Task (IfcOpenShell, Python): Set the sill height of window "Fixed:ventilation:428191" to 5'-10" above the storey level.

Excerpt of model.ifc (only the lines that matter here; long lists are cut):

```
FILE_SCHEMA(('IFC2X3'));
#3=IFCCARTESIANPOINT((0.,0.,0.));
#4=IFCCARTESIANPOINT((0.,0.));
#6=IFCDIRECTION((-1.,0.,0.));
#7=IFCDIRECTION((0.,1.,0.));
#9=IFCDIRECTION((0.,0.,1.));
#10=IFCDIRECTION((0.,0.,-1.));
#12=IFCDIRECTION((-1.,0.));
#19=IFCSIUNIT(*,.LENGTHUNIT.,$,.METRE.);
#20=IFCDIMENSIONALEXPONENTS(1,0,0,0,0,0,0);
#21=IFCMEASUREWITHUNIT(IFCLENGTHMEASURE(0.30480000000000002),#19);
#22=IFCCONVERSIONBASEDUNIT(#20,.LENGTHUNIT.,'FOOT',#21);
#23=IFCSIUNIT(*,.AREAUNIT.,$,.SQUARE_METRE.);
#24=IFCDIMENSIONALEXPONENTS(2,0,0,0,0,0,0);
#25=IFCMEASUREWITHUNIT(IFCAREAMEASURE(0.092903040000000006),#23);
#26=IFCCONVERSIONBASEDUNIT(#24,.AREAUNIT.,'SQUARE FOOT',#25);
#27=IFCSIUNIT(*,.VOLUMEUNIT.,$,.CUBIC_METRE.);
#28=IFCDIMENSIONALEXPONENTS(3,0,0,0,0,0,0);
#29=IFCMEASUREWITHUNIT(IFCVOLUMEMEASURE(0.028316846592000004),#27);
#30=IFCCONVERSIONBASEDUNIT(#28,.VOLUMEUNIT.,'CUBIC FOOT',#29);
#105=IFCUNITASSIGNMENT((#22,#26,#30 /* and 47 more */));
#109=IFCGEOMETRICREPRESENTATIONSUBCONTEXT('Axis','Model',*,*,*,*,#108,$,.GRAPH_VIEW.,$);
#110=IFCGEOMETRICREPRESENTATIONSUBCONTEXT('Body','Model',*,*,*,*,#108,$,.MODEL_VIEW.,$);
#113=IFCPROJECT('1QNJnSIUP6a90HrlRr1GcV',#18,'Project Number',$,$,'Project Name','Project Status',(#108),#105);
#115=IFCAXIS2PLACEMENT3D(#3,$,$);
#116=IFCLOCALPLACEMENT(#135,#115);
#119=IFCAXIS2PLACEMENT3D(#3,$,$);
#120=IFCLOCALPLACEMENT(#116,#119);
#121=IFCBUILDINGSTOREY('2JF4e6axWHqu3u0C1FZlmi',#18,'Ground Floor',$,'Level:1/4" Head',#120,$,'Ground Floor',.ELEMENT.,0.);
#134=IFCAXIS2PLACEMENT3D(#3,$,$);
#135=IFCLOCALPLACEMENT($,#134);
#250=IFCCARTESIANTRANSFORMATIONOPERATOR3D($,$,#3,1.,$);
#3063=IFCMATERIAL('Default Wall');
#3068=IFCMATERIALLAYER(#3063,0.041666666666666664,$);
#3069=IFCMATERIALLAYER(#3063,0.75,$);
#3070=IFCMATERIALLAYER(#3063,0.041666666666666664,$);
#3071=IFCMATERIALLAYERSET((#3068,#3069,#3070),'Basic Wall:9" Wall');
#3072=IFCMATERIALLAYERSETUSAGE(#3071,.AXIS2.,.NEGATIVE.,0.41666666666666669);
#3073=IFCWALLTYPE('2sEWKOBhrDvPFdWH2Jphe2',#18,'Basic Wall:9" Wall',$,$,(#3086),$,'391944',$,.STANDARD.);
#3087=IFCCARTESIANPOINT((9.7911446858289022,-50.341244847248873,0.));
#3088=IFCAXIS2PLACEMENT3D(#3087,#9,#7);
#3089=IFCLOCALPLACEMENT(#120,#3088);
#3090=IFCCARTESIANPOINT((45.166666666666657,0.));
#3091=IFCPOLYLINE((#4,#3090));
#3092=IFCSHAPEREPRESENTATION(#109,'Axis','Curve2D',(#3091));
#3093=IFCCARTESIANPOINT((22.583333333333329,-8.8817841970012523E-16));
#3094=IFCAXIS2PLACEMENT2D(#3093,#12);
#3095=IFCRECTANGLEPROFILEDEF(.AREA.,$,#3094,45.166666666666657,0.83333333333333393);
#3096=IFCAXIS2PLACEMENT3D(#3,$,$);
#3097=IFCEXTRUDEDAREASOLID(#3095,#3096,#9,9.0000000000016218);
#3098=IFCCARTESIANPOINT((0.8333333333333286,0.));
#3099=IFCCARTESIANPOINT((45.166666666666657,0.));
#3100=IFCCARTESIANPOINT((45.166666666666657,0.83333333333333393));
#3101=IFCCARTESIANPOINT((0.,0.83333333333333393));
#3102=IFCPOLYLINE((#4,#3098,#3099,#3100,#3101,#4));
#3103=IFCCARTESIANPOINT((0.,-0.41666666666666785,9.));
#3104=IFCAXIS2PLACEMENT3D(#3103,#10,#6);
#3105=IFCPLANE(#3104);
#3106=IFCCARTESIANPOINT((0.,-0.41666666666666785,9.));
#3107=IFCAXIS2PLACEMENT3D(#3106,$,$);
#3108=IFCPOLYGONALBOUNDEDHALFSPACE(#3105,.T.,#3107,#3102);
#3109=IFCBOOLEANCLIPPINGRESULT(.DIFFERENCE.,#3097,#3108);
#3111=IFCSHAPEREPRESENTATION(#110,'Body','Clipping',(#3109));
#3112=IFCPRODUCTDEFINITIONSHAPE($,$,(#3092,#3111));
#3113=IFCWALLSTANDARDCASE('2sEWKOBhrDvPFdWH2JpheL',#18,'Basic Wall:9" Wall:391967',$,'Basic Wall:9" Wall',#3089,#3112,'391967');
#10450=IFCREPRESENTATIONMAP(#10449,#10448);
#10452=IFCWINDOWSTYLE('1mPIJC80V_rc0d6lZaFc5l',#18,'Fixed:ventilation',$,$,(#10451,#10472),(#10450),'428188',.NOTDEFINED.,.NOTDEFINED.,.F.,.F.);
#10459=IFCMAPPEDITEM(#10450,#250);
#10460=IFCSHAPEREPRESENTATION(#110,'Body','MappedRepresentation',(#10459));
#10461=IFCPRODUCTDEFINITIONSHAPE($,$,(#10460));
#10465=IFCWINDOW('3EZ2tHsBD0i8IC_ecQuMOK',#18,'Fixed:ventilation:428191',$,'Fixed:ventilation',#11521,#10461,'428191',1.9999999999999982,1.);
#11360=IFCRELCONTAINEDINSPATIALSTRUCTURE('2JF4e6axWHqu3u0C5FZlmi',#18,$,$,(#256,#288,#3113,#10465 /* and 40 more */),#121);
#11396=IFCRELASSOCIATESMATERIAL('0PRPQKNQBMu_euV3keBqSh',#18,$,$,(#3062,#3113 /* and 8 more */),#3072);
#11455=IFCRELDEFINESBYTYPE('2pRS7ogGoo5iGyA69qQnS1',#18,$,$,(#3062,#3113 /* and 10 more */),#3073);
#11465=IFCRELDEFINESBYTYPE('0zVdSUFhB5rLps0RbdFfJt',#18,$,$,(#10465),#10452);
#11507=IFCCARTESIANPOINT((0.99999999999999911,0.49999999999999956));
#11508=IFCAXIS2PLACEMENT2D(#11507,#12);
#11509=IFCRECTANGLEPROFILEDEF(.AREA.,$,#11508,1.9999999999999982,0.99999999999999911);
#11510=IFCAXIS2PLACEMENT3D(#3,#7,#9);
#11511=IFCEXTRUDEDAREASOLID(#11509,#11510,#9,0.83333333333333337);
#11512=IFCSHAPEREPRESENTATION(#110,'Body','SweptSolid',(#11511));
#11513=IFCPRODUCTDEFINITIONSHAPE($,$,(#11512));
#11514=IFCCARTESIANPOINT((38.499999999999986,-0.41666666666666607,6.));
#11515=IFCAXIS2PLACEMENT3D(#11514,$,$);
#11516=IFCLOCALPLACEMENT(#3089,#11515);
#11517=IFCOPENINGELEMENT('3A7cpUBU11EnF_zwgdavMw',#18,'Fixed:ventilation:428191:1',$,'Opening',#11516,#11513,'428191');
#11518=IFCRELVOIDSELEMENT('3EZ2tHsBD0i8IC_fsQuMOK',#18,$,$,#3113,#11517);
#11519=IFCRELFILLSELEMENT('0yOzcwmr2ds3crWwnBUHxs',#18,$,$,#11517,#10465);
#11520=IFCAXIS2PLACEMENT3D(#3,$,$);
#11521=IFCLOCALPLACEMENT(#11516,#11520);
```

```python
import numpy as np
import ifcopenshell
import ifcopenshell.api.geometry
import ifcopenshell.geom
import ifcopenshell.util.element
import ifcopenshell.util.placement
import ifcopenshell.util.shape
import ifcopenshell.util.unit

model = ifcopenshell.open("model.ifc")
unit_scale = ifcopenshell.util.unit.calculate_unit_scale(model)

window = model.by_guid("3EZ2tHsBD0i8IC_ecQuMOK")
opening = window.FillsVoids[0].RelatingOpeningElement
storey = ifcopenshell.util.element.get_container(window, ifc_class="IfcBuildingStorey")
level = ifcopenshell.util.placement.get_local_placement(storey.ObjectPlacement)[2, 3]

# The opening's origin need not be at the sill, so measure its lowest point.
shape = ifcopenshell.geom.create_shape(ifcopenshell.geom.settings(), opening)
bottom = ifcopenshell.util.shape.get_shape_bottom_elevation(shape, shape.geometry) / unit_scale
dz = level + 70 * 0.0254 / unit_scale - bottom

shift = np.array([0.0, 0.0, dz])
# The window is placed relative to its opening, so it follows when the opening moves.
matrix = ifcopenshell.util.placement.get_local_placement(opening.ObjectPlacement)
matrix[:3, 3] += shift
ifcopenshell.api.geometry.edit_object_placement(
    model, product=opening, matrix=matrix, is_si=False, should_transform_children=True
)

print(f"moved by {dz * unit_scale:+.3f} m")

model.write("model_v2.ifc")
```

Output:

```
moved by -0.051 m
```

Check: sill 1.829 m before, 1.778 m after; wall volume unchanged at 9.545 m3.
